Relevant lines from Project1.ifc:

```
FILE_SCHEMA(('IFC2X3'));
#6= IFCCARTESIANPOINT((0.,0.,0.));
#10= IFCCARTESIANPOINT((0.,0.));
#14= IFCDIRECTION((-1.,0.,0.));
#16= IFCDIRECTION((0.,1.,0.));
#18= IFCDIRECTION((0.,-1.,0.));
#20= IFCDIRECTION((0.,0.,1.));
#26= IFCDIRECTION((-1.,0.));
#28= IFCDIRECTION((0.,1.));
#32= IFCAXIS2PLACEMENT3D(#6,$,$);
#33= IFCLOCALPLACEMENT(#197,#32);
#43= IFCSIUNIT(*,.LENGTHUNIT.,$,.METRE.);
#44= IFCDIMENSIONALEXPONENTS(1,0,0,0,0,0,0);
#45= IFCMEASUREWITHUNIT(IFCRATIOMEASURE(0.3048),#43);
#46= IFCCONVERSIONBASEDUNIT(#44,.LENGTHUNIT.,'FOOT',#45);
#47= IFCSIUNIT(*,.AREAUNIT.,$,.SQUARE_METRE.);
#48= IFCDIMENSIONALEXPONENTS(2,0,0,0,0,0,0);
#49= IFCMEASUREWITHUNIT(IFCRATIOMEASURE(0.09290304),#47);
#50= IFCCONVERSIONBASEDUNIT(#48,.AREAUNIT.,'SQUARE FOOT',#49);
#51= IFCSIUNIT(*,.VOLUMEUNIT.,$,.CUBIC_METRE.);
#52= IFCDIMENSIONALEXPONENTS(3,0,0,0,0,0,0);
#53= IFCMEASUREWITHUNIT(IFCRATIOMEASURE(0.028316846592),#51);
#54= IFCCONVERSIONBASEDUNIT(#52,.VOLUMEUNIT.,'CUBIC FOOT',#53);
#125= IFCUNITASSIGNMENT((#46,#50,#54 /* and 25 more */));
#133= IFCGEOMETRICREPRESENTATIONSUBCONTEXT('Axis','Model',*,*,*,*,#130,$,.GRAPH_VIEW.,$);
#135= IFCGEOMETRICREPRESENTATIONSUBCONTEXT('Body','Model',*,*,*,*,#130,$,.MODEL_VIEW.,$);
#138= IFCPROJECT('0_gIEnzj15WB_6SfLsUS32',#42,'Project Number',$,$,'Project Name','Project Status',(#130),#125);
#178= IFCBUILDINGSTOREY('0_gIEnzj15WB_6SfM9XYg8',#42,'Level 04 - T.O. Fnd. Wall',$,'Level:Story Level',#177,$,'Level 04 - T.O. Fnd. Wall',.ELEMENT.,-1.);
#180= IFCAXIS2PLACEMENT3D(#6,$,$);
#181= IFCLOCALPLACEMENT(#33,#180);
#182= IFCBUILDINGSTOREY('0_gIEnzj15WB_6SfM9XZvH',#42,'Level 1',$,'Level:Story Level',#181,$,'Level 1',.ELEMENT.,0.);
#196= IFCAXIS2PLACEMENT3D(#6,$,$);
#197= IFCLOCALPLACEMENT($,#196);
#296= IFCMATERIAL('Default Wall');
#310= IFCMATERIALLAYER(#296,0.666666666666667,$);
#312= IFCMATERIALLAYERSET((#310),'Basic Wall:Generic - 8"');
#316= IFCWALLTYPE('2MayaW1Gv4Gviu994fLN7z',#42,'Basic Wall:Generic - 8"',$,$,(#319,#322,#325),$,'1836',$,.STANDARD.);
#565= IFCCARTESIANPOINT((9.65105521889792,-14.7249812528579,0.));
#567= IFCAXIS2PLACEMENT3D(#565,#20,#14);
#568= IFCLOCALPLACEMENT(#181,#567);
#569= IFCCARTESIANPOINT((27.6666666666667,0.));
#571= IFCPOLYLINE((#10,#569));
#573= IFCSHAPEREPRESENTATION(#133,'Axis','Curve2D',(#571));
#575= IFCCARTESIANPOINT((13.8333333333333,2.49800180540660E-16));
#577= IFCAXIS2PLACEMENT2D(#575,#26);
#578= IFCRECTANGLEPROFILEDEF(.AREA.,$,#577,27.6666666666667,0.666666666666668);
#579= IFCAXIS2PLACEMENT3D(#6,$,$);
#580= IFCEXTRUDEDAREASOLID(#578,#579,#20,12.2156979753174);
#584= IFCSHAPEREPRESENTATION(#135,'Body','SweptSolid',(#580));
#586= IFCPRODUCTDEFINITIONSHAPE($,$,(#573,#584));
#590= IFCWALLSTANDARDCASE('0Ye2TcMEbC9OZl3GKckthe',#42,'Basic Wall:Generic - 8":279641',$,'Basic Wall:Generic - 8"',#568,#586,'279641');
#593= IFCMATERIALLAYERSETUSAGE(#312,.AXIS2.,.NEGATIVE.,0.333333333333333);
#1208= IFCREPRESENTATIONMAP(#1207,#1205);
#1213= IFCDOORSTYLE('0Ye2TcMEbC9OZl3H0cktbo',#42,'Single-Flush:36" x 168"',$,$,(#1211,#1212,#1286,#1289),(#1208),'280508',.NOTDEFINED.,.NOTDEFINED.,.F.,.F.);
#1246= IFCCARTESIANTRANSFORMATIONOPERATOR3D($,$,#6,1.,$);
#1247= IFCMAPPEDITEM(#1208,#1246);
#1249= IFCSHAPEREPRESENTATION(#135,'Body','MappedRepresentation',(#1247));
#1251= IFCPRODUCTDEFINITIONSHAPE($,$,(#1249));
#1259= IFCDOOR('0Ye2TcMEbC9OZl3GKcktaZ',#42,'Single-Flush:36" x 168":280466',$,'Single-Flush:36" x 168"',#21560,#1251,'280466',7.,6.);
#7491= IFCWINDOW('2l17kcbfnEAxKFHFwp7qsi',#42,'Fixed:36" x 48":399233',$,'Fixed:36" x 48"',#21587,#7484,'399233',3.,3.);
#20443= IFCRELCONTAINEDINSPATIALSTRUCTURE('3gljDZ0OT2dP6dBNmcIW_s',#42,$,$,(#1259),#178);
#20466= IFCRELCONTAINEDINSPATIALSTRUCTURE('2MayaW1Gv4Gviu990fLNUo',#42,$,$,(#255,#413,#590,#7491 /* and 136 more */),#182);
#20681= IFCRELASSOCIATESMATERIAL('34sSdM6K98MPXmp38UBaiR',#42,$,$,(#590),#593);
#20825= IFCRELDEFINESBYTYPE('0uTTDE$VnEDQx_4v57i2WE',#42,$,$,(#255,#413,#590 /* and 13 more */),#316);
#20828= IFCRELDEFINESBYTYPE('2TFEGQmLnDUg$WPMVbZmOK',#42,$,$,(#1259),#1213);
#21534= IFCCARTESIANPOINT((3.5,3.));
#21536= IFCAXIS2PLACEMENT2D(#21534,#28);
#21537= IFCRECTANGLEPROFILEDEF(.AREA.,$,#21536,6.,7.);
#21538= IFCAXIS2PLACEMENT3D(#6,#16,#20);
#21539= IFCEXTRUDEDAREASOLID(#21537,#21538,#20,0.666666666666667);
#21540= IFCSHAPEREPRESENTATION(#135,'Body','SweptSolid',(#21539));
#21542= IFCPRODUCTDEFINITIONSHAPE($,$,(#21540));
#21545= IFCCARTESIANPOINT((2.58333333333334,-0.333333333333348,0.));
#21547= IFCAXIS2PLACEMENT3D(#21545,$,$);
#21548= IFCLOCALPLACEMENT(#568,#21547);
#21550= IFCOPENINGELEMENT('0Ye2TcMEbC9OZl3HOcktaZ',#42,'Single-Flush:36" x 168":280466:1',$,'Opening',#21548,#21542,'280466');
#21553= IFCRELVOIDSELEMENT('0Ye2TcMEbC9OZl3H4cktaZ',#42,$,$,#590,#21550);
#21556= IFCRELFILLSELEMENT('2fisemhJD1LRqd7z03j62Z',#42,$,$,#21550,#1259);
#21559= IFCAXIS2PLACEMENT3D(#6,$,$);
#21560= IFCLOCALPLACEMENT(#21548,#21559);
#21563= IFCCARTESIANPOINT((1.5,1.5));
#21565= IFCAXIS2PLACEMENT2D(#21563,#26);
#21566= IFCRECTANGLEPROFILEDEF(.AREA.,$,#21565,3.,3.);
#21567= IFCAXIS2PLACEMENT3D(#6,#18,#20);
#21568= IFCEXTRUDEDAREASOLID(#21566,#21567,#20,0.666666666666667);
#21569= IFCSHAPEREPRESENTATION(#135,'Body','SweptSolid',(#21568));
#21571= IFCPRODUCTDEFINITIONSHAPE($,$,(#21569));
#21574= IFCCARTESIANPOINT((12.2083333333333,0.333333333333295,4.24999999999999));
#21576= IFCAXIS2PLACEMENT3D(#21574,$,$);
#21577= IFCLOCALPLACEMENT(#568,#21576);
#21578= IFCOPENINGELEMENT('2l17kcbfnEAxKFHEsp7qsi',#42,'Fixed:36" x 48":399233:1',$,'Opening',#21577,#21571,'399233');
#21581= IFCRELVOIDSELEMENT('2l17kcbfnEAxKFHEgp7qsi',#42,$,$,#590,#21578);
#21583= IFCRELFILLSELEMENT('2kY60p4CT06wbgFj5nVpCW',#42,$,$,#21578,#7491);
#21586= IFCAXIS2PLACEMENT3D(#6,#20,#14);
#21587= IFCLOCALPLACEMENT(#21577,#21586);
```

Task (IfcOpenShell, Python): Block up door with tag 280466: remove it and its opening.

```python
import ifcopenshell
import ifcopenshell.api.feature
import ifcopenshell.api.root
import ifcopenshell.geom
import ifcopenshell.util.shape

model = ifcopenshell.open("Project1.ifc")
settings = ifcopenshell.geom.settings()


def volume(element):
    """Net volume in cubic metres, openings subtracted."""
    shape = ifcopenshell.geom.create_shape(settings, element)
    return ifcopenshell.util.shape.get_volume(shape.geometry)


door = model.by_id(1259)
opening = door.FillsVoids[0].RelatingOpeningElement
wall = opening.VoidsElements[0].RelatingBuildingElement
before = volume(wall)

ifcopenshell.api.root.remove_product(model, product=door)
ifcopenshell.api.feature.remove_feature(model, feature=opening)

after = volume(wall)

print(f"wall volume {before:.3f} -> {after:.3f} m3")

model.write("Project1_edited.ifc")
```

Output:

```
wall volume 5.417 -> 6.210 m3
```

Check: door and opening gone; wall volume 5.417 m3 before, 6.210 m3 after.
